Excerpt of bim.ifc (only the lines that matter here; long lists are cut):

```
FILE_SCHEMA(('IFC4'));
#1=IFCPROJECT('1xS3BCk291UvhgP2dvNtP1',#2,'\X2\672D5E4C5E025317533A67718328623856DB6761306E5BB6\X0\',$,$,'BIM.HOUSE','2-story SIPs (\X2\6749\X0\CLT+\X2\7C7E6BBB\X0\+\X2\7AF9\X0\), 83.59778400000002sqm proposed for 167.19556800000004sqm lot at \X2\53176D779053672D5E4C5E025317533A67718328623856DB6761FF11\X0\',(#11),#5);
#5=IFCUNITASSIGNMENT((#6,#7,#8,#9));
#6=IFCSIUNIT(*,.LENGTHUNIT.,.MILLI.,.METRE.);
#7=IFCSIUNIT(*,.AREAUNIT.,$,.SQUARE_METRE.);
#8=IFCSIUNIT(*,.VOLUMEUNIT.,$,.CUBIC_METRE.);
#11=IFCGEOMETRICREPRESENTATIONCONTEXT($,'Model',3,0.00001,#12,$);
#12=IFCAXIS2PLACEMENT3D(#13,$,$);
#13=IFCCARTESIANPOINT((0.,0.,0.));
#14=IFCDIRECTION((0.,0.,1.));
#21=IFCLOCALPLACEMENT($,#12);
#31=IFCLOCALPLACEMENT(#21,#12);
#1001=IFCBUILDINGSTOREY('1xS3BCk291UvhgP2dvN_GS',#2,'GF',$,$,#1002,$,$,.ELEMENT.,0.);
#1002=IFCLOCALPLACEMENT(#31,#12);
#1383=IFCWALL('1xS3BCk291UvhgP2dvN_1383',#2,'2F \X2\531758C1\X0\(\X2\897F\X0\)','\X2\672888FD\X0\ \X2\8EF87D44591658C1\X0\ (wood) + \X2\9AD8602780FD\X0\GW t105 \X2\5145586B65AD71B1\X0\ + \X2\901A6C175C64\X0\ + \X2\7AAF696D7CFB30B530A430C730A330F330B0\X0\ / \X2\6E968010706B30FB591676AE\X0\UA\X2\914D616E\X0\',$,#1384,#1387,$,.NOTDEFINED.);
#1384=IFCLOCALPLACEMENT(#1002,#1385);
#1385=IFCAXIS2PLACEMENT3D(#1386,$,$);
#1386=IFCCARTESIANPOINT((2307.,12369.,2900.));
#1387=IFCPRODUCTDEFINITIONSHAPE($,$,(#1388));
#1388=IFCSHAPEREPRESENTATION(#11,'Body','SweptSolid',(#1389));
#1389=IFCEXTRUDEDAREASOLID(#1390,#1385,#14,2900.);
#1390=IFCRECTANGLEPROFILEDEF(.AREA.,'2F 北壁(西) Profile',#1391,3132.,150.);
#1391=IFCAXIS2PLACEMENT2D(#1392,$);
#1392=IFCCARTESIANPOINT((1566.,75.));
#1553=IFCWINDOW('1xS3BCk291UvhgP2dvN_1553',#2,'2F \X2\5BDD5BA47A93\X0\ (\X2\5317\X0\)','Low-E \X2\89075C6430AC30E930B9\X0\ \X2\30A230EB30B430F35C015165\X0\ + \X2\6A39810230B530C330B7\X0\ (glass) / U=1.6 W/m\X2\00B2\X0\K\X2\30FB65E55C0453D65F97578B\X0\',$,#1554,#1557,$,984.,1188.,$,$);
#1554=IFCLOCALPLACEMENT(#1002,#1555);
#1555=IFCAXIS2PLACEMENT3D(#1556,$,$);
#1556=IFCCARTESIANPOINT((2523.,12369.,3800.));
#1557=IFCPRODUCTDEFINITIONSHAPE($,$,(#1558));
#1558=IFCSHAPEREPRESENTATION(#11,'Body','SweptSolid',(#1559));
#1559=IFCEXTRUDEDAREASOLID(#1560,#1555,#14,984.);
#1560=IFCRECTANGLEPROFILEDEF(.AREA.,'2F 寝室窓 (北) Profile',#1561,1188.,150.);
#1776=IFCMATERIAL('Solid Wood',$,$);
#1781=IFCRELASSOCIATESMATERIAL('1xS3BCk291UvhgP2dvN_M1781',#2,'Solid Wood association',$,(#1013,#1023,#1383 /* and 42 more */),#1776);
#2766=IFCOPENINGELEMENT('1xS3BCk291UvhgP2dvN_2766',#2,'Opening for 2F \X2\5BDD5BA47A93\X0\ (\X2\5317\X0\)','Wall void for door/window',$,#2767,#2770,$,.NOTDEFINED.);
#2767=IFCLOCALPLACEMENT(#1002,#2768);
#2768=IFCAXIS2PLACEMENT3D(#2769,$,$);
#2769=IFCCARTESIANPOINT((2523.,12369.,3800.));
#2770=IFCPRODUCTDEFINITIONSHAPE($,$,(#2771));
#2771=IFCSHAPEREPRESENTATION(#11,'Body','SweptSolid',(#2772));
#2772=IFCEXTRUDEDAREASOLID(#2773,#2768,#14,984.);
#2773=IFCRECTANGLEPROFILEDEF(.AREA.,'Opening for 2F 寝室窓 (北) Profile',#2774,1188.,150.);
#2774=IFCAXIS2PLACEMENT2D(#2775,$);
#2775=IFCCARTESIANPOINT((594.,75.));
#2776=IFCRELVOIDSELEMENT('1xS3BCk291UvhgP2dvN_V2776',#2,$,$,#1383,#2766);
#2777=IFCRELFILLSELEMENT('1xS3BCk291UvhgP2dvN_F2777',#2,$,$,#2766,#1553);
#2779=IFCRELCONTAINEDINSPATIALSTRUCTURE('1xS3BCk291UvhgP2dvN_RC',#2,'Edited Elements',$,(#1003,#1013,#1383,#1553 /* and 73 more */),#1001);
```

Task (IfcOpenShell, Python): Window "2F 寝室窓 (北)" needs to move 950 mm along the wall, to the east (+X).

```python
import ifcopenshell
import ifcopenshell.api.geometry
import ifcopenshell.util.placement

model = ifcopenshell.open("bim.ifc")

window = model.by_guid("1xS3BCk291UvhgP2dvN_1553")
opening = window.FillsVoids[0].RelatingOpeningElement
wall = opening.VoidsElements[0].RelatingBuildingElement

wall_matrix = ifcopenshell.util.placement.get_local_placement(wall.ObjectPlacement)
shift = wall_matrix[:3, 0] * 950.0
before = ifcopenshell.util.placement.get_local_placement(window.ObjectPlacement)[:3, 3].copy()

# The window is not placed relative to its opening, so move both.
for product in (opening, window):
    matrix = ifcopenshell.util.placement.get_local_placement(product.ObjectPlacement)
    matrix[:3, 3] += shift
    ifcopenshell.api.geometry.edit_object_placement(model, product=product, matrix=matrix, is_si=False)

after = ifcopenshell.util.placement.get_local_placement(window.ObjectPlacement)[:3, 3]
print("window moved by", (after - before).round(3) + 0.0)

model.write("bim-out.ifc")
```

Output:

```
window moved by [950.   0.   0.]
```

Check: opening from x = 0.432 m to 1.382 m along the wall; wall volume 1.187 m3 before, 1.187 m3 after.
